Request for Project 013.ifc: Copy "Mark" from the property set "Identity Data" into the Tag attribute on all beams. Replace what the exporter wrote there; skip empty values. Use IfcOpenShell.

First a look at what the model holds.

```python
import ifcopenshell
import ifcopenshell.util.element

model = ifcopenshell.open("Project 013.ifc")
print(model.schema)
beams = model.by_type("IfcBeam")
print(len(beams), "beams")
for e in beams[:8]:
    source = ifcopenshell.util.element.get_pset(e, "Identity Data", "Mark")
    target = e.Tag
    print(e.id(), repr(source), repr(target), sep=" | ")
```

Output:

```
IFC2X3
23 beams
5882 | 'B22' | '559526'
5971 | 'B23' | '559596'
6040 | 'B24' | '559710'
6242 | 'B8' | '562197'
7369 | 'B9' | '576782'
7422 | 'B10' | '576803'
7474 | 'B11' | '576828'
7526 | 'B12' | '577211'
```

```python
import ifcopenshell
import ifcopenshell.util.element

model = ifcopenshell.open("Project 013.ifc")

count = 0
for e in model.by_type("IfcBeam"):
    value = ifcopenshell.util.element.get_pset(e, "Identity Data", "Mark")
    current = e.Tag
    if not value or not value.strip() or current == value:
        continue
    e.Tag = value
    count += 1

print(count, "beams updated")

model.write("Project 013_v2.ifc")
```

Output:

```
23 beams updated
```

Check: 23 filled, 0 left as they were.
